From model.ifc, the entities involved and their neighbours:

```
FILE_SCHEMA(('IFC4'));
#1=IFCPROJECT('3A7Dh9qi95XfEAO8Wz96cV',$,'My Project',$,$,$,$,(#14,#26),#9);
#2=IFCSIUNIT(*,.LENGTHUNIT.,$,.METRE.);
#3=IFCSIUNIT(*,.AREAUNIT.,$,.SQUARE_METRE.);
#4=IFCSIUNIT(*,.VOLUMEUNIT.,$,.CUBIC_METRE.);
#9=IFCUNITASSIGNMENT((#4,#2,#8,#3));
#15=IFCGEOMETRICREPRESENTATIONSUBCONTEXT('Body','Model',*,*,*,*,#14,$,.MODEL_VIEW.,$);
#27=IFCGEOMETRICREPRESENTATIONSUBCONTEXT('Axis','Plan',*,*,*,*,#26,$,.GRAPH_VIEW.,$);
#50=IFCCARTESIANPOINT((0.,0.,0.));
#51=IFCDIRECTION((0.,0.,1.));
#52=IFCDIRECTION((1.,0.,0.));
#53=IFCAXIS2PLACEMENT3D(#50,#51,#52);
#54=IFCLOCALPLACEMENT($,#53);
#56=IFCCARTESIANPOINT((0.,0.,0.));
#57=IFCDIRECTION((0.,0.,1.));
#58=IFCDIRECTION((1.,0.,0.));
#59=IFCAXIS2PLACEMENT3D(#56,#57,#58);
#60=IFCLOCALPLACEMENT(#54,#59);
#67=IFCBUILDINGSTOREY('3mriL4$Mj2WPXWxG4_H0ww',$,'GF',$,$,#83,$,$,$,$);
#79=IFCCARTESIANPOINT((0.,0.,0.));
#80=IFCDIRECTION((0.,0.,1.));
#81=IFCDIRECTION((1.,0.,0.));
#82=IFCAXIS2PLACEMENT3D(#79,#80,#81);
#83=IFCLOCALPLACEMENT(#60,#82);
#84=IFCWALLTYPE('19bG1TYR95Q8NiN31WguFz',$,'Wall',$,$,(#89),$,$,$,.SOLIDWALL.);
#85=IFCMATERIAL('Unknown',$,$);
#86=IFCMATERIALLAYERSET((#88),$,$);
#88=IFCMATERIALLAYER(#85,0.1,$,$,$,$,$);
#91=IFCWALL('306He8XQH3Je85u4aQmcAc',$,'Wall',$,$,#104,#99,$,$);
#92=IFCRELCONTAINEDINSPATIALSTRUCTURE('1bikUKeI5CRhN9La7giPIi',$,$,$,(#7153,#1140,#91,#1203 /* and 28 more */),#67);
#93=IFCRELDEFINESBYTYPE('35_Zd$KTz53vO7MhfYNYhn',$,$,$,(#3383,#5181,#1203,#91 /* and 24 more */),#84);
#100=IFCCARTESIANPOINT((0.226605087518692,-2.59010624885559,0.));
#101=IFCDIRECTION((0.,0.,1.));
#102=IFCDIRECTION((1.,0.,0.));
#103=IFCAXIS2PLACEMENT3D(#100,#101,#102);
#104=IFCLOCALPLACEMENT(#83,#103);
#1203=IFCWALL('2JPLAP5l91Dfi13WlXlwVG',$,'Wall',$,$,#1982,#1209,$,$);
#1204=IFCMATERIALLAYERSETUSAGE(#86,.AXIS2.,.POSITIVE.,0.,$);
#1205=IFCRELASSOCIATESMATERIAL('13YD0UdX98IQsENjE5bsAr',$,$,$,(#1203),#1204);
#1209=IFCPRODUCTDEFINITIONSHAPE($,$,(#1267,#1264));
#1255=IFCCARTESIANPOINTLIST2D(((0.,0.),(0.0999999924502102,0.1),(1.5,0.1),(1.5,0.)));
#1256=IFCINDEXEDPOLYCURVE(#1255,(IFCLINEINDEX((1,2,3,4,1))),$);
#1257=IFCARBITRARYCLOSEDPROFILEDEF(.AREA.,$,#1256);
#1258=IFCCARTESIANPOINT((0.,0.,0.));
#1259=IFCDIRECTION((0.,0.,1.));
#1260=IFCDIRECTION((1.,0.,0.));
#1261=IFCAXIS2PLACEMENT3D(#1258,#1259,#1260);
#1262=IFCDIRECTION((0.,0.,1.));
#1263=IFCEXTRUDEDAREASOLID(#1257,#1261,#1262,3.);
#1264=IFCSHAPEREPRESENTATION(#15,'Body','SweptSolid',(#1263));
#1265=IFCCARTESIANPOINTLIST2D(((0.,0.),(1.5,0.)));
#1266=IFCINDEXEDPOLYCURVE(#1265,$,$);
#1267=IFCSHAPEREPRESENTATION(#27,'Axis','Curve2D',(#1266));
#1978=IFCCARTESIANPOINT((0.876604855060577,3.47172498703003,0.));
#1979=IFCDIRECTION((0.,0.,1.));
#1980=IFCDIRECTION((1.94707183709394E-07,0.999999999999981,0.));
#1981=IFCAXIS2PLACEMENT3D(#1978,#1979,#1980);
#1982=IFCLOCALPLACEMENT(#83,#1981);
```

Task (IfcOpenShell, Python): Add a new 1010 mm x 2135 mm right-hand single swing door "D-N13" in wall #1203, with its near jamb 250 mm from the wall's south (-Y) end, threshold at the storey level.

```python
import numpy as np
import ifcopenshell
import ifcopenshell.api.feature
import ifcopenshell.api.geometry
import ifcopenshell.api.root
import ifcopenshell.api.spatial
import ifcopenshell.geom
import ifcopenshell.util.element
import ifcopenshell.util.placement
import ifcopenshell.util.representation
import ifcopenshell.util.shape
import ifcopenshell.util.unit

model = ifcopenshell.open("model.ifc")
unit_scale = ifcopenshell.util.unit.calculate_unit_scale(model)
settings = ifcopenshell.geom.settings()


def volume(element):
    """Net volume in cubic metres, openings subtracted."""
    shape = ifcopenshell.geom.create_shape(settings, element)
    return ifcopenshell.util.shape.get_volume(shape.geometry)


wall = model.by_guid("2JPLAP5l91Dfi13WlXlwVG")
storey = ifcopenshell.util.element.get_container(wall, ifc_class="IfcBuildingStorey")
context = ifcopenshell.util.representation.get_context(model, "Model", "Body", "MODEL_VIEW")
before = volume(wall)

width, height, from_end, sill = 1.01, 2.135, 0.25, 0.0  # metres

# The wall runs along its own X axis, and the end named is its -X end.
wall_shape = ifcopenshell.geom.create_shape(settings, wall)
x, y, z = ifcopenshell.util.shape.get_vertices(wall_shape.geometry).T
start = x.min() + from_end
face, thickness = float(y.min()), float(y.max() - y.min())
wall_matrix = ifcopenshell.util.placement.get_local_placement(wall.ObjectPlacement)
level = ifcopenshell.util.placement.get_local_placement(storey.ObjectPlacement)[2, 3]


def in_wall(x, y):
    """Placement at x, y metres in the wall's axes, at sill height."""
    matrix = wall_matrix.copy()
    matrix[:, 3] = wall_matrix @ np.array([x / unit_scale, y / unit_scale, 0.0, 1.0])
    matrix[2, 3] = level + sill / unit_scale
    return matrix


# Opening: a box that overshoots both wall faces by 50 mm.
opening = ifcopenshell.api.root.create_entity(model, ifc_class="IfcOpeningElement", predefined_type="OPENING")
box = ifcopenshell.api.geometry.add_wall_representation(
    model, context=context, length=width, height=height, thickness=thickness + 0.1
)
ifcopenshell.api.geometry.assign_representation(model, product=opening, representation=box)
ifcopenshell.api.geometry.edit_object_placement(model, product=opening, matrix=in_wall(start, face - 0.05), is_si=False)
ifcopenshell.api.feature.add_feature(model, feature=opening, element=wall)

door = ifcopenshell.api.root.create_entity(model, ifc_class="IfcDoor", name="D-N13", predefined_type="DOOR")
door.OverallWidth, door.OverallHeight = width / unit_scale, height / unit_scale
door.OperationType = "SINGLE_SWING_RIGHT"
body = ifcopenshell.api.geometry.add_door_representation(
    model,
    context=context,
    overall_width=door.OverallWidth,
    overall_height=door.OverallHeight,
    operation_type="SINGLE_SWING_RIGHT",
    lining_properties={"LiningDepth": thickness / unit_scale, "ThresholdDepth": thickness / unit_scale},
)
ifcopenshell.api.geometry.assign_representation(model, product=door, representation=body)
ifcopenshell.api.spatial.assign_container(model, products=[door], relating_structure=storey)
ifcopenshell.api.feature.add_filling(model, opening=opening, element=door)

# The lining spans the wall, so the door starts at the wall face.
ifcopenshell.api.geometry.edit_object_placement(model, product=door, matrix=in_wall(start, face), is_si=False)

after = volume(wall)

print(f"wall volume {before:.3f} -> {after:.3f} m3")

model.write("model_updated.ifc")
```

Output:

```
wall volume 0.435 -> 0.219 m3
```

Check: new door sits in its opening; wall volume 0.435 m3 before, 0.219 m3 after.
